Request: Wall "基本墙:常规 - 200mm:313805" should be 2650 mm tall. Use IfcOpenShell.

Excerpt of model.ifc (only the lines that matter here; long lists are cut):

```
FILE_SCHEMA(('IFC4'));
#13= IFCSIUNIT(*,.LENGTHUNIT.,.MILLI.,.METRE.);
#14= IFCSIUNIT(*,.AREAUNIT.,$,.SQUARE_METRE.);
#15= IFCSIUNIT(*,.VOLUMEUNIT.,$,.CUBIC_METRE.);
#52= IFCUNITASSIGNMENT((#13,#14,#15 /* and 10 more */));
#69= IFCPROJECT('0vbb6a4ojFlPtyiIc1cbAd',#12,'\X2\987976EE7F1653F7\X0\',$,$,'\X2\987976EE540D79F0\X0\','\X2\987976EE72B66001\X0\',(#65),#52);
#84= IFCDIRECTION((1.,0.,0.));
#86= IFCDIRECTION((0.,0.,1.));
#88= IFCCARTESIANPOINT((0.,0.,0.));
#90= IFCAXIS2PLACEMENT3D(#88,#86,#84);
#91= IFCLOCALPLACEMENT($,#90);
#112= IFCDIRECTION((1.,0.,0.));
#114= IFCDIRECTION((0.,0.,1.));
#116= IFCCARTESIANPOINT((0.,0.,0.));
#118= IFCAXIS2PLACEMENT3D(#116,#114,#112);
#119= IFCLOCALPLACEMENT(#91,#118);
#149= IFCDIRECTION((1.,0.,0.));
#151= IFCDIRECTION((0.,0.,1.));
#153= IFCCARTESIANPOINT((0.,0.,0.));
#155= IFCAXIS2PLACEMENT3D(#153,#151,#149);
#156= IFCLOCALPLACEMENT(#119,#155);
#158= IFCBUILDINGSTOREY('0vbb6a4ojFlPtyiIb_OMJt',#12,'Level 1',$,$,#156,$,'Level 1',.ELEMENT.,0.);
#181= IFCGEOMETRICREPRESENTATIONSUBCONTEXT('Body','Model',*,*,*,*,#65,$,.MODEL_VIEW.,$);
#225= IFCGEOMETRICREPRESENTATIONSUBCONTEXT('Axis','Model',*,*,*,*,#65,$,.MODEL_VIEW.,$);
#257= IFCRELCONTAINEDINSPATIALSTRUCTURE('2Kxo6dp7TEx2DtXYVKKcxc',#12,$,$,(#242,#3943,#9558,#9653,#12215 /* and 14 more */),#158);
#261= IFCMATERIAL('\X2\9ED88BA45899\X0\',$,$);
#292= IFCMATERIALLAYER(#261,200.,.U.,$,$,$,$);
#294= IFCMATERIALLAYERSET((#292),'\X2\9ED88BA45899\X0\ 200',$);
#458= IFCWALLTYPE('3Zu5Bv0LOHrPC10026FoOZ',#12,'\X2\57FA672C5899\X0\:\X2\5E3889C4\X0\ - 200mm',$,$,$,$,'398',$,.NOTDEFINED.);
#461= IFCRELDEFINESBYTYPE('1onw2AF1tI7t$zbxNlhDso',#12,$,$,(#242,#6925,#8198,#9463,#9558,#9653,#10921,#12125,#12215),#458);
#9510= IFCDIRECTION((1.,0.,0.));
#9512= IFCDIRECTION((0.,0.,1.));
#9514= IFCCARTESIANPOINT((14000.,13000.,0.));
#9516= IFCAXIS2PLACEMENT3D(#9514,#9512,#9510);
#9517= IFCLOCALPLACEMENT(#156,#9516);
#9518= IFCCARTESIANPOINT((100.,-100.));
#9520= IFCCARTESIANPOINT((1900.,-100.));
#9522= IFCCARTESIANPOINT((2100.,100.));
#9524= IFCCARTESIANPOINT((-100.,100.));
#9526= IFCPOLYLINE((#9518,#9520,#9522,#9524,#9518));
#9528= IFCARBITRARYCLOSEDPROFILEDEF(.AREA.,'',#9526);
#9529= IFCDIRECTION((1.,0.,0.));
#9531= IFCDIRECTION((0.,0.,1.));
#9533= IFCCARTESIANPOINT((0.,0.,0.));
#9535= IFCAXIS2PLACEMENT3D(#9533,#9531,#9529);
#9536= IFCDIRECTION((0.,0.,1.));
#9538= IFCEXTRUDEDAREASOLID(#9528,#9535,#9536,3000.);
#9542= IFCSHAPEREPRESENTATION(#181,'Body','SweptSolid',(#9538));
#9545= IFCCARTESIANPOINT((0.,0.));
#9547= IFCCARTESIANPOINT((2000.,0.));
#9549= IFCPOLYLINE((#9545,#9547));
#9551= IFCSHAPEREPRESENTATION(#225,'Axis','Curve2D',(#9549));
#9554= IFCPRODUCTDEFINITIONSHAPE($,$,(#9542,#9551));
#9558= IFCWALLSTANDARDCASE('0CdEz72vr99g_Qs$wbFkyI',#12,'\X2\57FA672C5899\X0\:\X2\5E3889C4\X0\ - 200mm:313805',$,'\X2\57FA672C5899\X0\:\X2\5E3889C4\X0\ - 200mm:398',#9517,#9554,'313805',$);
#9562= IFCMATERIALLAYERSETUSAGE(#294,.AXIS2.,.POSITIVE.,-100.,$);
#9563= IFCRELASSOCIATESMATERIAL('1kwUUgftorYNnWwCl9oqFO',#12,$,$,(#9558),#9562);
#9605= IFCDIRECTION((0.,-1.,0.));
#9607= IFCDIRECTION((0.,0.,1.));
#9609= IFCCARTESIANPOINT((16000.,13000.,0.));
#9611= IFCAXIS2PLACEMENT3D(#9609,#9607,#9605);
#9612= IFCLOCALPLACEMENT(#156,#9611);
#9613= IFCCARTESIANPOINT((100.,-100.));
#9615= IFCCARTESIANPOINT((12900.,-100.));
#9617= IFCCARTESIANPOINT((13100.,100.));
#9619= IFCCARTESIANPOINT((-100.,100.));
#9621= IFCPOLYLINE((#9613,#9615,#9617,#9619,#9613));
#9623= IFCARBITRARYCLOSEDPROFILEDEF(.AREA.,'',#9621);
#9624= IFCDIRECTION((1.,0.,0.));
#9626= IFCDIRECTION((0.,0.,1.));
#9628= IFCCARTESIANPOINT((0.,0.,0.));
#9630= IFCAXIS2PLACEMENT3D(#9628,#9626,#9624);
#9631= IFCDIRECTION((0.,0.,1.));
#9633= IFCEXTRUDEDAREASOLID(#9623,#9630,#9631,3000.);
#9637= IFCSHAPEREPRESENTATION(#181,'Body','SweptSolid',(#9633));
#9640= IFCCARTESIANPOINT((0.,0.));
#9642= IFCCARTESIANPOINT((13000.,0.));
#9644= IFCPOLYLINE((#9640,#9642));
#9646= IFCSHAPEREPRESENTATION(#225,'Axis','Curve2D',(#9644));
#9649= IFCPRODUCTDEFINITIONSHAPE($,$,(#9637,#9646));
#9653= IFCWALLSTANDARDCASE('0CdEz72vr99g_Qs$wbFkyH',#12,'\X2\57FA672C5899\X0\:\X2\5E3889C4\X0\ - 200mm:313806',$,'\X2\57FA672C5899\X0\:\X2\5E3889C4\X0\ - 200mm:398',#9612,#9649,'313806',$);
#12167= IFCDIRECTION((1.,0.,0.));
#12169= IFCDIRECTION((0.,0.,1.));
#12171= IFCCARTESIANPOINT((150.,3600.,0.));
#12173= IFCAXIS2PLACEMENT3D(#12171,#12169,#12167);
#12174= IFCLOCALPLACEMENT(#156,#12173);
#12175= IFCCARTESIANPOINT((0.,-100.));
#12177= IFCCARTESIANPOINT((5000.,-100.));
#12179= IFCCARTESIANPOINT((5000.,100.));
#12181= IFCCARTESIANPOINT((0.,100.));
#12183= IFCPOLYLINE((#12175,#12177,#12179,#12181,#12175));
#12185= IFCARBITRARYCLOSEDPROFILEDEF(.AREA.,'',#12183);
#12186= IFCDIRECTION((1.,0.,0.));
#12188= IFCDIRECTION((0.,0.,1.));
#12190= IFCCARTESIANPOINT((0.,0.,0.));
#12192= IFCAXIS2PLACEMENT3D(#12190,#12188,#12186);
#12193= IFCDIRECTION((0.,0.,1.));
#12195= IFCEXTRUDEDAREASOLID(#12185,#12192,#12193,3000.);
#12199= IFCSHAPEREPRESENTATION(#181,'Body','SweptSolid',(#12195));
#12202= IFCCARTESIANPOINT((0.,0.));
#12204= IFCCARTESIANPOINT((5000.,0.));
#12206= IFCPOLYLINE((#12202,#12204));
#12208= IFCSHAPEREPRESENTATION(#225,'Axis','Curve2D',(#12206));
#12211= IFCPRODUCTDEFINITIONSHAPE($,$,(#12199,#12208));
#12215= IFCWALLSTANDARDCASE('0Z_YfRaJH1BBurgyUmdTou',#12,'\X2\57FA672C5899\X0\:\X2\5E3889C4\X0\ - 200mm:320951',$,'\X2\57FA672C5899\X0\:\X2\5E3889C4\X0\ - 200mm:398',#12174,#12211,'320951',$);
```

```python
import ifcopenshell
import ifcopenshell.geom
import ifcopenshell.util.representation
import ifcopenshell.util.shape
import ifcopenshell.util.unit

model = ifcopenshell.open("model.ifc")
unit_scale = ifcopenshell.util.unit.calculate_unit_scale(model)
settings = ifcopenshell.geom.settings()


def volume(element):
    """Net volume in cubic metres, openings subtracted."""
    shape = ifcopenshell.geom.create_shape(settings, element)
    return ifcopenshell.util.shape.get_volume(shape.geometry)


wall = model.by_guid("0CdEz72vr99g_Qs$wbFkyI")
before = volume(wall)

body = ifcopenshell.util.representation.get_representation(wall, "Model", "Body")
solid = body.Items[0]
old_height = solid.Depth
solid.Depth = 2.65 / unit_scale
after = volume(wall)

print(f"height {old_height:g} -> {solid.Depth:g}, volume {before:.3f} -> {after:.3f} m3")

model.write("model_v2.ifc")
```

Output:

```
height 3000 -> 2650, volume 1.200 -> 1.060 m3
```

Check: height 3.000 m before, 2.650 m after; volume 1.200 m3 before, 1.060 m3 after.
